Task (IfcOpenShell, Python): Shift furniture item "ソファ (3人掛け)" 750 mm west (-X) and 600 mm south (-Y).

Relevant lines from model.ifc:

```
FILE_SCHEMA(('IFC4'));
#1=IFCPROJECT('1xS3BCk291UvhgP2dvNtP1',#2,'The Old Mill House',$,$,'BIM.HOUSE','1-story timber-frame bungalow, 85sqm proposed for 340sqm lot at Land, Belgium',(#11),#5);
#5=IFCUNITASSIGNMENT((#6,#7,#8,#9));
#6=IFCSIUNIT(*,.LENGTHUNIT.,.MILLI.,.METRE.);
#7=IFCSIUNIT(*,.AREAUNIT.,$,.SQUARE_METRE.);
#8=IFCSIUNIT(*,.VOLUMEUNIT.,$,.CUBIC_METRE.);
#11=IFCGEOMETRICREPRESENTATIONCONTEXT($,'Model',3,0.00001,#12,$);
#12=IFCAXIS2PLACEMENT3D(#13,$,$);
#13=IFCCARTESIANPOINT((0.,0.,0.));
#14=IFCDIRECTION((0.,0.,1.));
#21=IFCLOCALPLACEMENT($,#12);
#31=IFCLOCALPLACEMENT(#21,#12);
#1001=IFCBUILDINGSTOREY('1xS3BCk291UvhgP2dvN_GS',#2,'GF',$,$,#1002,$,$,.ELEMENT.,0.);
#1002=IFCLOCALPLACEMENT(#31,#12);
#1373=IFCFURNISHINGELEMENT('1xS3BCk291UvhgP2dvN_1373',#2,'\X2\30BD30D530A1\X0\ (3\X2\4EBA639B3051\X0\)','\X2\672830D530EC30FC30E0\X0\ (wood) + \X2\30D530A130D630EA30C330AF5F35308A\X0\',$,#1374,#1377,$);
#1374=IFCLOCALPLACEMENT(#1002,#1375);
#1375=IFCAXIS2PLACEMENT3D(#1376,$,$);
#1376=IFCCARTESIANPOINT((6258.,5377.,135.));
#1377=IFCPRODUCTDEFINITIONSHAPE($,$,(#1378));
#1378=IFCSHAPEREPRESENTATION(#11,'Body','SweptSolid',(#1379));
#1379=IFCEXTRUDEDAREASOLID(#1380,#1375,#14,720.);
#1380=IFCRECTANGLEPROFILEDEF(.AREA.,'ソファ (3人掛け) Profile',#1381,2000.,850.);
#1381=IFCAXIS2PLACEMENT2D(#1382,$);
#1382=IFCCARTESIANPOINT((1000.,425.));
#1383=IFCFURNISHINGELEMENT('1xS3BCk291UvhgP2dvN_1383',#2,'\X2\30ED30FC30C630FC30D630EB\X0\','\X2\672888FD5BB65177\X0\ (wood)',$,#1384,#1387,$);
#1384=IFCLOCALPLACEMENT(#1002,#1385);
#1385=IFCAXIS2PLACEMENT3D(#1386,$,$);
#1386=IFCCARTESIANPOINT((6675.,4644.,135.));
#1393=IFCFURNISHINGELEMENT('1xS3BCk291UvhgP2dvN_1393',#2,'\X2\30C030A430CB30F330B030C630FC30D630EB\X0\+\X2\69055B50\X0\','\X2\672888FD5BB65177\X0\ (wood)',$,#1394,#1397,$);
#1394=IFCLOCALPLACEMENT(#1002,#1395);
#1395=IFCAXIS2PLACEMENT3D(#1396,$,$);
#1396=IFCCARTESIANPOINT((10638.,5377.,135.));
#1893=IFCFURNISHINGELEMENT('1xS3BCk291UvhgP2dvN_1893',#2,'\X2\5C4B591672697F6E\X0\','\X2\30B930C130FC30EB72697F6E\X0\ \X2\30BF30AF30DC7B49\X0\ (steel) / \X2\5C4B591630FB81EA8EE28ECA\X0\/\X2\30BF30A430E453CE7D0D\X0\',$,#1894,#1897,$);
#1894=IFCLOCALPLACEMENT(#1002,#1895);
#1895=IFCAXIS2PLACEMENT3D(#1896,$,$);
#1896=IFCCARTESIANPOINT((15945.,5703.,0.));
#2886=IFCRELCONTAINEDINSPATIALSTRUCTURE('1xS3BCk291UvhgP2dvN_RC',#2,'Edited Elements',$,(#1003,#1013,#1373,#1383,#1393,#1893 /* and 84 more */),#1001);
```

```python
import ifcopenshell
import ifcopenshell.api.geometry
import ifcopenshell.util.placement
import ifcopenshell.util.unit

model = ifcopenshell.open("model.ifc")
unit_scale = ifcopenshell.util.unit.calculate_unit_scale(model)

item = model.by_guid("1xS3BCk291UvhgP2dvN_1373")
matrix = ifcopenshell.util.placement.get_local_placement(item.ObjectPlacement)
matrix[0, 3] -= 0.75 / unit_scale
matrix[1, 3] -= 0.6 / unit_scale
ifcopenshell.api.geometry.edit_object_placement(model, product=item, matrix=matrix, is_si=False)

print(ifcopenshell.util.placement.get_local_placement(item.ObjectPlacement).round(3) + 0.0)

model.write("model_v2.ifc")
```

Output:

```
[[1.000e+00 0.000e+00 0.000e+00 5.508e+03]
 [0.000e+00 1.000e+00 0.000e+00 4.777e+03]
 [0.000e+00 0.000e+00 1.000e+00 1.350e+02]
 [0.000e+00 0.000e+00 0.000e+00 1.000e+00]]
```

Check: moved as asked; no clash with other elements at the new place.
